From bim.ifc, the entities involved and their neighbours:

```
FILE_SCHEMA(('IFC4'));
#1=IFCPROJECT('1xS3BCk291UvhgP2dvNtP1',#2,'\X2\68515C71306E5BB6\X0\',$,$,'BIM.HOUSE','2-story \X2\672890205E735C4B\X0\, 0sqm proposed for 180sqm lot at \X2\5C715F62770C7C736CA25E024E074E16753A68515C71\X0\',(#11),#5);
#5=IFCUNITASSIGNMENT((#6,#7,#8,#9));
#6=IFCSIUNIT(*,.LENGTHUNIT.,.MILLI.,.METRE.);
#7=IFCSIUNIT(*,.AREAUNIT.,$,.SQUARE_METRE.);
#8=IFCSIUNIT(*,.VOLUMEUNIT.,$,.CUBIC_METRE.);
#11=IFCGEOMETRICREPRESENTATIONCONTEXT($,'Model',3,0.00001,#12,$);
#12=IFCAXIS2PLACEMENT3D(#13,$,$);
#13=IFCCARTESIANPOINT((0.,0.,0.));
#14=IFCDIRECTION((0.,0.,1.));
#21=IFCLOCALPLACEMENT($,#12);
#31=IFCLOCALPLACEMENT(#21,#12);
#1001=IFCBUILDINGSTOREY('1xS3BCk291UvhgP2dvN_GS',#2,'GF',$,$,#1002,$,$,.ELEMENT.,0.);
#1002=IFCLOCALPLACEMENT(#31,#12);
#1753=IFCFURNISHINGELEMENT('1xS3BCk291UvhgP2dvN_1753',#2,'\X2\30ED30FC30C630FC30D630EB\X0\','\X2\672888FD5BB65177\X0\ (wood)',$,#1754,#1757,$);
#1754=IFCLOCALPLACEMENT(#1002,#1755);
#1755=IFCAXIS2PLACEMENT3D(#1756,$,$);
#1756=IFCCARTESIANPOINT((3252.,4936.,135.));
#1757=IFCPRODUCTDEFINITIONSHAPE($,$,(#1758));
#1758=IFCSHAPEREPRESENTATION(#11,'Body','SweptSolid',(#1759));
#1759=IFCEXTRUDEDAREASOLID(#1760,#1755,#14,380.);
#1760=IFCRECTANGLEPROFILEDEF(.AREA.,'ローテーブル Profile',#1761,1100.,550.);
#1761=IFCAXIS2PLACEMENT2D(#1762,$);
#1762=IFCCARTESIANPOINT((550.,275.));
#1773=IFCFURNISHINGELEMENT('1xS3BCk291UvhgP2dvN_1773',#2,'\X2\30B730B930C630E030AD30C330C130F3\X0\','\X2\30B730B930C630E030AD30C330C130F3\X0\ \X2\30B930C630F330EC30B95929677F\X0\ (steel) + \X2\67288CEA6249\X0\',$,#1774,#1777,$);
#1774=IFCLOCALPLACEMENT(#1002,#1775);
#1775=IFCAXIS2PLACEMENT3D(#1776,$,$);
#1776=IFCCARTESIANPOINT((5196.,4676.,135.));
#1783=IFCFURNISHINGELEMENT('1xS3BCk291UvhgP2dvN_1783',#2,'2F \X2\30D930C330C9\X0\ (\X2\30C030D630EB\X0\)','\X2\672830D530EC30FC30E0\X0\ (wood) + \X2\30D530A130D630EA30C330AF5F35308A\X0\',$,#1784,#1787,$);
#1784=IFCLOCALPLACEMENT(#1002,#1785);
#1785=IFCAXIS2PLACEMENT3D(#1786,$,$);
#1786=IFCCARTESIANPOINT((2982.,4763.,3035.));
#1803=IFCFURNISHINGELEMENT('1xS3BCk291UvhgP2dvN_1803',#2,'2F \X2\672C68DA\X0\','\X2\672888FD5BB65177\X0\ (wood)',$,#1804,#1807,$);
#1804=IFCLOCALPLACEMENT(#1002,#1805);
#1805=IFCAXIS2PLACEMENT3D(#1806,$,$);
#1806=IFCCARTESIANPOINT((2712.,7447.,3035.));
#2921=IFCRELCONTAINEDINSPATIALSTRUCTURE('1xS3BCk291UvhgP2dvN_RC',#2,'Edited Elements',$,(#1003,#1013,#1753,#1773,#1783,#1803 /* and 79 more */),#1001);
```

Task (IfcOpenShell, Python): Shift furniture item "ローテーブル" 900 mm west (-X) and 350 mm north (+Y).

```python
import ifcopenshell
import ifcopenshell.api.geometry
import ifcopenshell.util.placement
import ifcopenshell.util.unit

model = ifcopenshell.open("bim.ifc")
unit_scale = ifcopenshell.util.unit.calculate_unit_scale(model)

item = model.by_guid("1xS3BCk291UvhgP2dvN_1753")
matrix = ifcopenshell.util.placement.get_local_placement(item.ObjectPlacement)
matrix[0, 3] -= 0.9 / unit_scale
matrix[1, 3] += 0.35 / unit_scale
ifcopenshell.api.geometry.edit_object_placement(model, product=item, matrix=matrix, is_si=False)

print(ifcopenshell.util.placement.get_local_placement(item.ObjectPlacement).round(3) + 0.0)

model.write("bim_rev.ifc")
```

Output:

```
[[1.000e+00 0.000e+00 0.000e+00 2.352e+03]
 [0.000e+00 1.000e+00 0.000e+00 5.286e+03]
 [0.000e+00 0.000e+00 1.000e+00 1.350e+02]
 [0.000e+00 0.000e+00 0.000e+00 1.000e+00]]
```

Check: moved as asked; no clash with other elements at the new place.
